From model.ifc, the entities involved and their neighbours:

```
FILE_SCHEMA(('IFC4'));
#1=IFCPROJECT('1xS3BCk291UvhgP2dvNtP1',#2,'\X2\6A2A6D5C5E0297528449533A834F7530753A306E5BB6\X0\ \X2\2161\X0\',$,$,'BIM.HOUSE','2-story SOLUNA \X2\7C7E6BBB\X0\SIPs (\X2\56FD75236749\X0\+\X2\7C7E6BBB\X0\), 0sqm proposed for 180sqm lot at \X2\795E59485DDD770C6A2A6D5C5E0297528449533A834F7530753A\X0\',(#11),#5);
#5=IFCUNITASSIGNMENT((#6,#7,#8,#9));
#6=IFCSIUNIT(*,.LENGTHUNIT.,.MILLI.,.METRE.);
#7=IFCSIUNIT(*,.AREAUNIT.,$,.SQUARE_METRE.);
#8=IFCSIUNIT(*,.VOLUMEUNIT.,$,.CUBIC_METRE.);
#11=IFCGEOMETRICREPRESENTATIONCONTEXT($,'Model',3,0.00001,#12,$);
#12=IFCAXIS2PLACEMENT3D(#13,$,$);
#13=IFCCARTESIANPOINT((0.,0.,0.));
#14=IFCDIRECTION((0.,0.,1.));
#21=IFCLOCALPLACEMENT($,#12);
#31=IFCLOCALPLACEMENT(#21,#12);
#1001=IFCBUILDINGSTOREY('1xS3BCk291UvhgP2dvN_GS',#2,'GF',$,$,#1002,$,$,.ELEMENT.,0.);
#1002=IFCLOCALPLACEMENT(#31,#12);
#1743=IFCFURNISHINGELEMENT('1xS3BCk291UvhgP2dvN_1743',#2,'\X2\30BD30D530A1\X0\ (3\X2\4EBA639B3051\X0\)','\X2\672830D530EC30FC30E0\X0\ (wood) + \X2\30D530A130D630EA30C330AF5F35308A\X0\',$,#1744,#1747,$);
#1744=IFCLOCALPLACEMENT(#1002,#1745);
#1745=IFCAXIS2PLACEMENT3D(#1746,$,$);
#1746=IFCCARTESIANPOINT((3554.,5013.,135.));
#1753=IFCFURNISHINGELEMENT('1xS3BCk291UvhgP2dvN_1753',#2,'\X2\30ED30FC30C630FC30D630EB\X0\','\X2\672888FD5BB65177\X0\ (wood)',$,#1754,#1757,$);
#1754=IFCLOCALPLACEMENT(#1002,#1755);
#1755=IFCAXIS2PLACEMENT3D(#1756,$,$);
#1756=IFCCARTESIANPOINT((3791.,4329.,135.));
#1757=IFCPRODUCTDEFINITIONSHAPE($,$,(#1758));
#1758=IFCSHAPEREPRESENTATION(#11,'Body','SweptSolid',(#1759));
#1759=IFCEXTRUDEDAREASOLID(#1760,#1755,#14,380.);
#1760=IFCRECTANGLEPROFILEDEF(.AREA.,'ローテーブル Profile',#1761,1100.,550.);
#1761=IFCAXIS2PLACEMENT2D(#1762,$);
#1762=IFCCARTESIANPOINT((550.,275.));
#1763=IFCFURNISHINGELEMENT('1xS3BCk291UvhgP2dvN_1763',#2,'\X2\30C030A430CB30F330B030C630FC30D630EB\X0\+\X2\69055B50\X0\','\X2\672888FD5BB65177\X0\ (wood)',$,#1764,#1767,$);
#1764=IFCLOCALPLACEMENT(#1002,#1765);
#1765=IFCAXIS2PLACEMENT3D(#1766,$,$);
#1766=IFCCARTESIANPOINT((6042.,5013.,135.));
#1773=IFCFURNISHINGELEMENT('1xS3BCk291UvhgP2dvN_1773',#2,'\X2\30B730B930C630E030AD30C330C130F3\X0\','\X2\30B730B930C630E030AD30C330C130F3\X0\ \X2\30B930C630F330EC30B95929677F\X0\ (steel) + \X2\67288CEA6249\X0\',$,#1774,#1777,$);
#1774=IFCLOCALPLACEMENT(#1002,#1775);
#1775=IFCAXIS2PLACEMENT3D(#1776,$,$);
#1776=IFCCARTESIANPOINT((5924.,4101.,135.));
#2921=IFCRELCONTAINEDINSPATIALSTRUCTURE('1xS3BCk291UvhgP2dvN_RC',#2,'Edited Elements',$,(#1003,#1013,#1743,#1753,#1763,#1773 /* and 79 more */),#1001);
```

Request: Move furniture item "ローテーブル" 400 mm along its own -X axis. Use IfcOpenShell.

```python
import ifcopenshell
import ifcopenshell.api.geometry
import ifcopenshell.util.placement

model = ifcopenshell.open("model.ifc")

item = model.by_guid("1xS3BCk291UvhgP2dvN_1753")
matrix = ifcopenshell.util.placement.get_local_placement(item.ObjectPlacement)
matrix[:3, 3] -= matrix[:3, 0] * 400.0
ifcopenshell.api.geometry.edit_object_placement(model, product=item, matrix=matrix, is_si=False)

print(ifcopenshell.util.placement.get_local_placement(item.ObjectPlacement).round(3) + 0.0)

model.write("model_updated.ifc")
```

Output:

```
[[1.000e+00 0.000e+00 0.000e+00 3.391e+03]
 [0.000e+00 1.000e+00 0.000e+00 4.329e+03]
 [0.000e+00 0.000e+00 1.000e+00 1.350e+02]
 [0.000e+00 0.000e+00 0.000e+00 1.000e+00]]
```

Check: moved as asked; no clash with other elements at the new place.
